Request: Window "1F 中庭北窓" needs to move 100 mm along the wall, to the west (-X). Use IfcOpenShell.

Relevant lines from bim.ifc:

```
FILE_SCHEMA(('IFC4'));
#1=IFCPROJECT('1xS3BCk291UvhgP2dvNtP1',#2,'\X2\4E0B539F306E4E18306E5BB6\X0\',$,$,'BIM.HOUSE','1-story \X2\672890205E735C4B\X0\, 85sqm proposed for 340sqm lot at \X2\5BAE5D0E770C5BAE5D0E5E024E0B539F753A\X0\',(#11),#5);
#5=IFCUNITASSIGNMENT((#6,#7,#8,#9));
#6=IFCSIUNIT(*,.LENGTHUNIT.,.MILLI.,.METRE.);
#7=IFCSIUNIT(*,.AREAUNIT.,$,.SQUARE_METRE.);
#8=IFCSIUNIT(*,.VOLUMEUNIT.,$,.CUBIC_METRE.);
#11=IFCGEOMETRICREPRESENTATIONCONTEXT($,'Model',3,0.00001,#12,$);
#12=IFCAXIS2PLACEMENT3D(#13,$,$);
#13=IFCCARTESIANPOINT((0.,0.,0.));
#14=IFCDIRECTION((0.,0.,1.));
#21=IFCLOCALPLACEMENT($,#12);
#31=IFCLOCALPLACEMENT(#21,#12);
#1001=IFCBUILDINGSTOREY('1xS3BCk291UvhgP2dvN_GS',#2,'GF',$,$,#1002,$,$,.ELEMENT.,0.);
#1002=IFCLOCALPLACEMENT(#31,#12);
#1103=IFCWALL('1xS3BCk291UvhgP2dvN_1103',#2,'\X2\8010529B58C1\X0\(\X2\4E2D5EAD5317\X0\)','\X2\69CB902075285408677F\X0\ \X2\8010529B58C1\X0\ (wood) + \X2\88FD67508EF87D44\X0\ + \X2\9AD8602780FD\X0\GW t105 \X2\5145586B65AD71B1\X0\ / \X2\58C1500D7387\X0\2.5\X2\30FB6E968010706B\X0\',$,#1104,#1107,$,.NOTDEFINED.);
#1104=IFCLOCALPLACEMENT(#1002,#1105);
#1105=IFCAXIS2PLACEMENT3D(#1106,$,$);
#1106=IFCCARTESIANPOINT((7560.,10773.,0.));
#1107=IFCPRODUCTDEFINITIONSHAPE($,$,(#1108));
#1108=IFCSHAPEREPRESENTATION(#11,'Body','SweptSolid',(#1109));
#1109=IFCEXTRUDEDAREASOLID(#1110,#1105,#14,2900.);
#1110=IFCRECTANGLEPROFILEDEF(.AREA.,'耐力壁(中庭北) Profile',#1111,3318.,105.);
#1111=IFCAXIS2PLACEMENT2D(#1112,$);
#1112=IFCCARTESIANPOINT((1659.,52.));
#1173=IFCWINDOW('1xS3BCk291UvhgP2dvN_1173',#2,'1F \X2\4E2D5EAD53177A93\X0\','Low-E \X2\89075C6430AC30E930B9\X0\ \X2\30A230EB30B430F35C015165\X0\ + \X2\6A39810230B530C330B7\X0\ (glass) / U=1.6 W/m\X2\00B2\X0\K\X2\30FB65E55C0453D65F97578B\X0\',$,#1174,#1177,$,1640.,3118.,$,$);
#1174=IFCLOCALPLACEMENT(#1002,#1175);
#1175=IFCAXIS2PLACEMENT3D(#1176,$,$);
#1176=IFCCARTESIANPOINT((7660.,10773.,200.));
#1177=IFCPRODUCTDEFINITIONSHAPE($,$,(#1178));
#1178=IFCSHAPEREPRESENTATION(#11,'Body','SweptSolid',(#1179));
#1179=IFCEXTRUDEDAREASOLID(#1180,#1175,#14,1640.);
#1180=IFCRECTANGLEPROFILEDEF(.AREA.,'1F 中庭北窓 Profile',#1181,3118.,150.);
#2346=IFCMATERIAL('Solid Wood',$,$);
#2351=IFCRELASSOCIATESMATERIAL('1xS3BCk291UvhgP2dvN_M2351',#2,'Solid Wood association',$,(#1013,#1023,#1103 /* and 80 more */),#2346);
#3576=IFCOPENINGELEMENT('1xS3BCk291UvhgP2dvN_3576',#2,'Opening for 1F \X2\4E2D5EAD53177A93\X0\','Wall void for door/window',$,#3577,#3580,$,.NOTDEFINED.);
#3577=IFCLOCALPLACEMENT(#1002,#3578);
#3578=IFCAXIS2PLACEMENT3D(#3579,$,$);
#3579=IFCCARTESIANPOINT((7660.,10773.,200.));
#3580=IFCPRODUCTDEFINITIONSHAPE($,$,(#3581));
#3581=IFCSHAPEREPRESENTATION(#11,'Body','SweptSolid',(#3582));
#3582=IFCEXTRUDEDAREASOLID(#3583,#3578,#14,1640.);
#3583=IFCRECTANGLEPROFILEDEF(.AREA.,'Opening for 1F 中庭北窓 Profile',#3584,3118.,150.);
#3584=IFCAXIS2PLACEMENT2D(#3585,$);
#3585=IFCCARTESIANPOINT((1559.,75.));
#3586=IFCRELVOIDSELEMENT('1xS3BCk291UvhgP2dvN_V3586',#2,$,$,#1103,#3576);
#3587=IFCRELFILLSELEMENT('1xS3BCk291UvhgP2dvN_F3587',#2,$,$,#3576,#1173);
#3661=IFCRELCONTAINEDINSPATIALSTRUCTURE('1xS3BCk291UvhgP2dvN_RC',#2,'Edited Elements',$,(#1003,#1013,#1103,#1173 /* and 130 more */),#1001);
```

```python
import ifcopenshell
import ifcopenshell.api.geometry
import ifcopenshell.util.placement

model = ifcopenshell.open("bim.ifc")

window = model.by_id(1173)
opening = window.FillsVoids[0].RelatingOpeningElement
wall = opening.VoidsElements[0].RelatingBuildingElement

wall_matrix = ifcopenshell.util.placement.get_local_placement(wall.ObjectPlacement)
shift = wall_matrix[:3, 0] * -100.0
before = ifcopenshell.util.placement.get_local_placement(window.ObjectPlacement)[:3, 3].copy()

# The window is not placed relative to its opening, so move both.
for product in (opening, window):
    matrix = ifcopenshell.util.placement.get_local_placement(product.ObjectPlacement)
    matrix[:3, 3] += shift
    ifcopenshell.api.geometry.edit_object_placement(model, product=product, matrix=matrix, is_si=False)

after = ifcopenshell.util.placement.get_local_placement(window.ObjectPlacement)[:3, 3]
print("window moved by", (after - before).round(3) + 0.0)

model.write("bim_updated.ifc")
```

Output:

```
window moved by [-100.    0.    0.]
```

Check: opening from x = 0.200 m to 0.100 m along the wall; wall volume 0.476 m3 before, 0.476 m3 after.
